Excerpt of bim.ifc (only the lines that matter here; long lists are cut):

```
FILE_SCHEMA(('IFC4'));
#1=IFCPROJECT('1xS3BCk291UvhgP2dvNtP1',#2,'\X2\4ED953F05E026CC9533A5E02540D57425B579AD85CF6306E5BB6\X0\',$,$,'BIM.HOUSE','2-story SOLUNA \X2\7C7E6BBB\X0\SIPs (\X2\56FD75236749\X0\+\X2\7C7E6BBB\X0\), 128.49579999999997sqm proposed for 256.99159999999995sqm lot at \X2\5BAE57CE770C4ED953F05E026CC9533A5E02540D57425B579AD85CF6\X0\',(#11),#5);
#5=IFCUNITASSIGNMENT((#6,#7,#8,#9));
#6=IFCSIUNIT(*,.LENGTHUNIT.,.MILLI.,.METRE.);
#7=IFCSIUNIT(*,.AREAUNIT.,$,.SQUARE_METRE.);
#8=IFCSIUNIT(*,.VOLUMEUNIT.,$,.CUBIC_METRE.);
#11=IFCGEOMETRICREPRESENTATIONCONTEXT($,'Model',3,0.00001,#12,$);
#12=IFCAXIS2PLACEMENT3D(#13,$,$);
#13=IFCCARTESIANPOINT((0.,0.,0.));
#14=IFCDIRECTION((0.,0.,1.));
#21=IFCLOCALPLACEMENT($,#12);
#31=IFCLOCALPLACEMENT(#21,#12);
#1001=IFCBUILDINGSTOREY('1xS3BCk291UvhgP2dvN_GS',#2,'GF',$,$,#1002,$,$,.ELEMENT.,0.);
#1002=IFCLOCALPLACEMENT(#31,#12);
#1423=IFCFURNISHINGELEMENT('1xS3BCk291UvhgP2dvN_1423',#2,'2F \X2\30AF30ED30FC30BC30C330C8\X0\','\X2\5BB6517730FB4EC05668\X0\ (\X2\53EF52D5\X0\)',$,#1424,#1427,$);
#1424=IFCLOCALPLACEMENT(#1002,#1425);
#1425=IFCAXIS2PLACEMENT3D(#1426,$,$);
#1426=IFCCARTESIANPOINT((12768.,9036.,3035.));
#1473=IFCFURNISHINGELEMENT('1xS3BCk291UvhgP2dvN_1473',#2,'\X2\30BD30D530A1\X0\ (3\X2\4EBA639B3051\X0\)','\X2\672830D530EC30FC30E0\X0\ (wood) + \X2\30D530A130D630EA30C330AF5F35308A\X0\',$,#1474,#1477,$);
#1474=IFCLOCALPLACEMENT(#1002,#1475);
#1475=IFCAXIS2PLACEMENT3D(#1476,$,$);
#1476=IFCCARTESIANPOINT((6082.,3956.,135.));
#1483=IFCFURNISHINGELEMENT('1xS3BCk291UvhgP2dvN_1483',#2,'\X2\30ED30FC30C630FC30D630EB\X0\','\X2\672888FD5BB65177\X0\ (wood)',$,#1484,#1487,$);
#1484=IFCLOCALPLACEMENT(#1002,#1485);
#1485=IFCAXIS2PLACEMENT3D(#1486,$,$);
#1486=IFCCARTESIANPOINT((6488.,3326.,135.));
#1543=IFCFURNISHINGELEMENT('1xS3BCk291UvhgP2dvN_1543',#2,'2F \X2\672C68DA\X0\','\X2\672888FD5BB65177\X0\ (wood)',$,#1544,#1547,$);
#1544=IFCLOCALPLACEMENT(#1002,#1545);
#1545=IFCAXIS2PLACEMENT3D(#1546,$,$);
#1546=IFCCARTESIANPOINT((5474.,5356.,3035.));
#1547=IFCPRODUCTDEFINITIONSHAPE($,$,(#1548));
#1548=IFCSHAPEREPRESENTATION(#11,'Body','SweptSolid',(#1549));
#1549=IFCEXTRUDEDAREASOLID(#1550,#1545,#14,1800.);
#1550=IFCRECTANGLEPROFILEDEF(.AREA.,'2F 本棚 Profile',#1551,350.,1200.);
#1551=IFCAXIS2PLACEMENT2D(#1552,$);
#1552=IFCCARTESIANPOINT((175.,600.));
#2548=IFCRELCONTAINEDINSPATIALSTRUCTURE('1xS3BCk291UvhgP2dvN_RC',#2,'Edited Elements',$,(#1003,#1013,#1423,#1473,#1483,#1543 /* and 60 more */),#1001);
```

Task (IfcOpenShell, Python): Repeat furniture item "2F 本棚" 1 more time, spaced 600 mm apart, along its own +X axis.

```python
import ifcopenshell
import ifcopenshell.api.geometry
import ifcopenshell.api.root
import ifcopenshell.util.element
import ifcopenshell.util.placement

model = ifcopenshell.open("bim.ifc")


def reuse_history(source, copy):
    """copy_class also copies each property set's owner history, people and application; keep the originals."""
    for rel in copy.IsDefinedBy:
        if rel.is_a("IfcRelDefinesByProperties") and (history := rel.RelatingPropertyDefinition.OwnerHistory):
            rel.RelatingPropertyDefinition.OwnerHistory = source.OwnerHistory
            ifcopenshell.util.element.remove_deep2(model, history)


source = model.by_guid("1xS3BCk291UvhgP2dvN_1543")
base = ifcopenshell.util.placement.get_local_placement(source.ObjectPlacement)
step = base[:3, 0] * 600.0

for i in range(1, 2):
    copy = ifcopenshell.api.root.copy_class(model, product=source)
    copy.Representation = ifcopenshell.util.element.copy_deep(
        model, source.Representation, exclude=["IfcGeometricRepresentationContext", "IfcRepresentationMap"]
    )
    reuse_history(source, copy)
    matrix = base.copy()
    matrix[:3, 3] += i * step
    print("added at", matrix[:3, 3].round(3) + 0.0)
    ifcopenshell.api.geometry.edit_object_placement(model, product=copy, matrix=matrix, is_si=False)

model.write("bim_updated.ifc")
```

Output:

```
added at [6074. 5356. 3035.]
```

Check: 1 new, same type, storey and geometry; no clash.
